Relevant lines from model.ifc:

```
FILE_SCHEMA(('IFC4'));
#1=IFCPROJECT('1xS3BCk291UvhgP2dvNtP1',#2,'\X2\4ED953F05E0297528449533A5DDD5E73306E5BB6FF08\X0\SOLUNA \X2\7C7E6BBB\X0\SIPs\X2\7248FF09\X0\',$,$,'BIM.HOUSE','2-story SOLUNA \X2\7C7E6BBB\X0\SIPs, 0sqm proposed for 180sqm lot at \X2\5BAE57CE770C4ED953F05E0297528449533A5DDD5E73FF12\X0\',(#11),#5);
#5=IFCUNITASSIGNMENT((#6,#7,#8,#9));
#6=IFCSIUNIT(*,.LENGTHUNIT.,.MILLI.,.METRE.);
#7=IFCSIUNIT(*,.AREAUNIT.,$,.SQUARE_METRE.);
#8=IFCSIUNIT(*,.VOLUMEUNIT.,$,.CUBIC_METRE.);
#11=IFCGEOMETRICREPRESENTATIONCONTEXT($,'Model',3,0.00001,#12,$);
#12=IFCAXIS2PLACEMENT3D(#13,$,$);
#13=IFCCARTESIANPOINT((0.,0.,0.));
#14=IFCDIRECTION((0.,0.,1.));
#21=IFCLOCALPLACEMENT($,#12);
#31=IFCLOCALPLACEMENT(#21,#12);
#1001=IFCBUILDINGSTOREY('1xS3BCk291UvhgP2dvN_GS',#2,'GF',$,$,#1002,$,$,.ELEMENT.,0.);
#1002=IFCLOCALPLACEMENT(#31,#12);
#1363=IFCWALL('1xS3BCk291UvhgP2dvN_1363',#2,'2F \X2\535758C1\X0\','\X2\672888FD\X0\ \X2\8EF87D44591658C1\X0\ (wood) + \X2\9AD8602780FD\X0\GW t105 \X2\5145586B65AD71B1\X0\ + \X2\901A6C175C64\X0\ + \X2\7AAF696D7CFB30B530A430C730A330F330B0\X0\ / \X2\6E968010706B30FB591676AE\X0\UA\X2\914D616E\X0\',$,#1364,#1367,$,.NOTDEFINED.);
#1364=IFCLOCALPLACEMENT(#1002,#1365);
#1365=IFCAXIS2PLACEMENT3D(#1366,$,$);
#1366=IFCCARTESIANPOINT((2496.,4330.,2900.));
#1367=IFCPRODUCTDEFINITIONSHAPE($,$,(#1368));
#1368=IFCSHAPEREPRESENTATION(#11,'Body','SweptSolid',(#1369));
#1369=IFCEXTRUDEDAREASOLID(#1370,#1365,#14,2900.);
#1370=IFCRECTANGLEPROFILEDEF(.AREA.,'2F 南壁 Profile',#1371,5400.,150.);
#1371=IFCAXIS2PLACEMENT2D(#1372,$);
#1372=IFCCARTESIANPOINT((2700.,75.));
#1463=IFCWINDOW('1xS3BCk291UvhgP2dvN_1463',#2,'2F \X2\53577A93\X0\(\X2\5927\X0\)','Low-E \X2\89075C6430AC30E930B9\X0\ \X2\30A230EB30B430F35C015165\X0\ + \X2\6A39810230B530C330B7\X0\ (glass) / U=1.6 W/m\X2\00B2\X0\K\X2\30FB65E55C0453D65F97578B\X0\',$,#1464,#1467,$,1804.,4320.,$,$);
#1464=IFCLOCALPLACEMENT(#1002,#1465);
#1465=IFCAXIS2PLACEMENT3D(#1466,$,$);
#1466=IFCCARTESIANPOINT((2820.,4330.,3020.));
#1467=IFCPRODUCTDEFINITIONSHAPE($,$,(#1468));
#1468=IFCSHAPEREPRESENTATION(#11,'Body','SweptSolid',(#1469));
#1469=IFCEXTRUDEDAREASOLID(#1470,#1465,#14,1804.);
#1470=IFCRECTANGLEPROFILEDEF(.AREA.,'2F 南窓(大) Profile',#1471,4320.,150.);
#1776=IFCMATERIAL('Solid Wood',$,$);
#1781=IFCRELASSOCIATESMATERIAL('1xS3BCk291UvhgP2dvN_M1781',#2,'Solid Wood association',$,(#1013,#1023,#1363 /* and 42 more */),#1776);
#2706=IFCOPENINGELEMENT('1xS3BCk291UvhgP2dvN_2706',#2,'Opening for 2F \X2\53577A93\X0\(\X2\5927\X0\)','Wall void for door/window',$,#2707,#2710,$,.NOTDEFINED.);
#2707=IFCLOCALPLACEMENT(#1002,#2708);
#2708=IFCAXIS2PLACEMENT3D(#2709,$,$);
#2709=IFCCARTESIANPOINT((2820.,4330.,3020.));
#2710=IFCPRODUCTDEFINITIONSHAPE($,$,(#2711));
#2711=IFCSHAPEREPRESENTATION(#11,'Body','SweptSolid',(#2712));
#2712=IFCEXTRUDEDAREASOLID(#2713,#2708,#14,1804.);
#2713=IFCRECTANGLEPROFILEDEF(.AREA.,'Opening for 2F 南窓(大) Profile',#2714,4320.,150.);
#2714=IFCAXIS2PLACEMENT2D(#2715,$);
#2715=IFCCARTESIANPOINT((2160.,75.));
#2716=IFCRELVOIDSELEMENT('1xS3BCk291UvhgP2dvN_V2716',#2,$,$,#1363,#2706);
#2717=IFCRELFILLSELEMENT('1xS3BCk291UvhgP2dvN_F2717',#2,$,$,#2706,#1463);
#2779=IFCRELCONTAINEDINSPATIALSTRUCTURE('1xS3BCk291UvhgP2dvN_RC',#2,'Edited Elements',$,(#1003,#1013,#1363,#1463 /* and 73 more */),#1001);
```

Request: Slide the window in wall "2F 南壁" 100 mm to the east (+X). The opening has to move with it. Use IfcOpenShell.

```python
import ifcopenshell
import ifcopenshell.api.geometry
import ifcopenshell.util.placement

model = ifcopenshell.open("model.ifc")

window = model.by_guid("1xS3BCk291UvhgP2dvN_1463")
opening = window.FillsVoids[0].RelatingOpeningElement
wall = opening.VoidsElements[0].RelatingBuildingElement

wall_matrix = ifcopenshell.util.placement.get_local_placement(wall.ObjectPlacement)
shift = wall_matrix[:3, 0] * 100.0
before = ifcopenshell.util.placement.get_local_placement(window.ObjectPlacement)[:3, 3].copy()

# The window is not placed relative to its opening, so move both.
for product in (opening, window):
    matrix = ifcopenshell.util.placement.get_local_placement(product.ObjectPlacement)
    matrix[:3, 3] += shift
    ifcopenshell.api.geometry.edit_object_placement(model, product=product, matrix=matrix, is_si=False)

after = ifcopenshell.util.placement.get_local_placement(window.ObjectPlacement)[:3, 3]
print("window moved by", (after - before).round(3) + 0.0)

model.write("model_rev.ifc")
```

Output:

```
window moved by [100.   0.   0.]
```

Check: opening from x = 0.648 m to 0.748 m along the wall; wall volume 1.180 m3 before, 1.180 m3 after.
